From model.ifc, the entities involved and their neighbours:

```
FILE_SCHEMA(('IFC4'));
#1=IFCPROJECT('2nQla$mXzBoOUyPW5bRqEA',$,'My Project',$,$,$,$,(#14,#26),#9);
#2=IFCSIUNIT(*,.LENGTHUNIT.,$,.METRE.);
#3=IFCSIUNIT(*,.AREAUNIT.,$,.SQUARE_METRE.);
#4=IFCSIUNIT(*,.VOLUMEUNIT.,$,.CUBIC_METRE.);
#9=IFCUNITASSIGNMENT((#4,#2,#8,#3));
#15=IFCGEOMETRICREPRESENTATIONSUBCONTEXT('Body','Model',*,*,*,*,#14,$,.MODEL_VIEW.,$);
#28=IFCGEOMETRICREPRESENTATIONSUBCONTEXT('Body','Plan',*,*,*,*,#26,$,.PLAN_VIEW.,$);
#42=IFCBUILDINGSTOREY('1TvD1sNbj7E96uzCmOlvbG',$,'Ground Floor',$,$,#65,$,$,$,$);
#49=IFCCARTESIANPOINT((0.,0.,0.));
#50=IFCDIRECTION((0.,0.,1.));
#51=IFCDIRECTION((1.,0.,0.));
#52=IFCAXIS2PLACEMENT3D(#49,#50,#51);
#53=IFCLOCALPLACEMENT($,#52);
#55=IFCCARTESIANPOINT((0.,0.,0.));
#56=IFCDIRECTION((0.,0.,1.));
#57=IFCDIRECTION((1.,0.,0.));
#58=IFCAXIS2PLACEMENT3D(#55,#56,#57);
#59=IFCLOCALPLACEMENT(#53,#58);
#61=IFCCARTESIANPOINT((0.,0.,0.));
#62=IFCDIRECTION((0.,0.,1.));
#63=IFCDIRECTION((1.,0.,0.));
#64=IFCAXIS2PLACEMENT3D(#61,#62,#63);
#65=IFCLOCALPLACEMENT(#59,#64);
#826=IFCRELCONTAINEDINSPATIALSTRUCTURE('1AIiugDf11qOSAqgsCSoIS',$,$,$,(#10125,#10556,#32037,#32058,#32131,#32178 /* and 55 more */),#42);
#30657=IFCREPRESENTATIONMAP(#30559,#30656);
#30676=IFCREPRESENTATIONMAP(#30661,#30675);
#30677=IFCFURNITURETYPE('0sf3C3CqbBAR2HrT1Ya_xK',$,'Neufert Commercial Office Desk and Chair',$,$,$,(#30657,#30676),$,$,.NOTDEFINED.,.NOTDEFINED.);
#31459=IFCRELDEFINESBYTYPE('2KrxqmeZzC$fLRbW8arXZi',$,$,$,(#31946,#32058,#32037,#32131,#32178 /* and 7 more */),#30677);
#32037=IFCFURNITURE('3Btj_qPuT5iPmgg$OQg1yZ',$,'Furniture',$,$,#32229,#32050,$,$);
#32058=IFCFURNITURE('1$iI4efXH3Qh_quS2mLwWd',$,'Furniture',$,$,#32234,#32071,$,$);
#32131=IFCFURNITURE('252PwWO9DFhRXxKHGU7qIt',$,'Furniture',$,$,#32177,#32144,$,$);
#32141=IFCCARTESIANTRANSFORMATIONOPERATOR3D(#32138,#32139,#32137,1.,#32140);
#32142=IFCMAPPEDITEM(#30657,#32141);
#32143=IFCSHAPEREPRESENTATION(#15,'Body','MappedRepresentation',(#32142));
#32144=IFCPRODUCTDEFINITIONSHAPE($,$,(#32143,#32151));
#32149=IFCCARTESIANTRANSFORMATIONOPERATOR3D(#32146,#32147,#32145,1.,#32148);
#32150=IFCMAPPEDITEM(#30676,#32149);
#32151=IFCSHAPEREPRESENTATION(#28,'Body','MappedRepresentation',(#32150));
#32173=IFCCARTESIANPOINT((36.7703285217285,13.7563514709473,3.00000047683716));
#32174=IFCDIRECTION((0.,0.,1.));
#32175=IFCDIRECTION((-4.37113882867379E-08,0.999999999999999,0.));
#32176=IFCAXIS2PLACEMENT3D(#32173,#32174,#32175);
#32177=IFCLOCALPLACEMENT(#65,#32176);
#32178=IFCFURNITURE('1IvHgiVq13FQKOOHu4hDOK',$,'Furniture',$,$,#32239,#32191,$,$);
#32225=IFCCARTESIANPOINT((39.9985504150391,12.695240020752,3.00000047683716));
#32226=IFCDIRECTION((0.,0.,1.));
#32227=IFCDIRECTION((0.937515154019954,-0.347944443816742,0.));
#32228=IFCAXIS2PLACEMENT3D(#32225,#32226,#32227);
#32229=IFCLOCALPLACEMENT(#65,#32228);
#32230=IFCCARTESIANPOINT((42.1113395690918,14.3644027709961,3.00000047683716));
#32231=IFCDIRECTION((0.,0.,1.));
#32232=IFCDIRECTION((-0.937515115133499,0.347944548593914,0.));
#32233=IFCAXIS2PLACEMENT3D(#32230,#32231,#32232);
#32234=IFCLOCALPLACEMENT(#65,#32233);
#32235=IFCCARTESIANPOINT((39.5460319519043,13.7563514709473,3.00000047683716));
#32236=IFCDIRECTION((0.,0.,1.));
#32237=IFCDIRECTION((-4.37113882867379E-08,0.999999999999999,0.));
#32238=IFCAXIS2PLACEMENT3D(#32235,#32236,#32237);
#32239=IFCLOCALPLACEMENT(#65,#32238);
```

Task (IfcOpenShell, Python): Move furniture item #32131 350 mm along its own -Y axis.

```python
import ifcopenshell
import ifcopenshell.api.geometry
import ifcopenshell.util.placement
import ifcopenshell.util.unit

model = ifcopenshell.open("model.ifc")
unit_scale = ifcopenshell.util.unit.calculate_unit_scale(model)

item = model.by_id(32131)
matrix = ifcopenshell.util.placement.get_local_placement(item.ObjectPlacement)
matrix[:3, 3] -= matrix[:3, 1] * 0.35 / unit_scale
ifcopenshell.api.geometry.edit_object_placement(model, product=item, matrix=matrix, is_si=False)

print(ifcopenshell.util.placement.get_local_placement(item.ObjectPlacement).round(3) + 0.0)

model.write("model_rev.ifc")
```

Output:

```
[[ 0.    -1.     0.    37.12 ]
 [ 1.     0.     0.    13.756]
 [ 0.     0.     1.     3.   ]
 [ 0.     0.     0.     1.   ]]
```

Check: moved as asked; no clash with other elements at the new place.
